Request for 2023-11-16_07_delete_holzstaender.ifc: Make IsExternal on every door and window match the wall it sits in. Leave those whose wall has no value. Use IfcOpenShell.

First a look at what the model holds.

```python
import ifcopenshell
import ifcopenshell.util.element

model = ifcopenshell.open("2023-11-16_07_delete_holzstaender.ifc")
print(model.schema)
seen = {}
for e in model.by_type("IfcDoor") + model.by_type("IfcWindow"):
    if not e.FillsVoids:
        continue
    host = e.FillsVoids[0].RelatingOpeningElement.VoidsElements[0].RelatingBuildingElement
    own = ifcopenshell.util.element.get_pset(e, f"Pset_{e.is_a()[3:].removesuffix('StandardCase')}Common", "IsExternal")
    wall = ifcopenshell.util.element.get_pset(host, "Pset_WallCommon", "IsExternal")
    seen[e.is_a(), own, wall] = seen.get((e.is_a(), own, wall), 0) + 1
for (cls, own, wall), count in sorted(seen.items(), key=str):
    print(count, cls, "IsExternal:", own, "| host wall:", wall)
```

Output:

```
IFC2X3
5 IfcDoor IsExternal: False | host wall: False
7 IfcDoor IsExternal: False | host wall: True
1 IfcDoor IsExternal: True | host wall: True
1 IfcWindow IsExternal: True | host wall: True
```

```python
import ifcopenshell
import ifcopenshell.api.pset
import ifcopenshell.util.element

model = ifcopenshell.open("2023-11-16_07_delete_holzstaender.ifc")

count = 0
for ifc_class, pset_name in (("IfcDoor", "Pset_DoorCommon"), ("IfcWindow", "Pset_WindowCommon")):
    for e in model.by_type(ifc_class):
        if not e.FillsVoids:
            continue
        host = e.FillsVoids[0].RelatingOpeningElement.VoidsElements[0].RelatingBuildingElement
        external = ifcopenshell.util.element.get_pset(host, "Pset_WallCommon", "IsExternal")
        if external is None or ifcopenshell.util.element.get_pset(e, pset_name, "IsExternal") == external:
            continue
        pset = ifcopenshell.api.pset.add_pset(model, product=e, name=pset_name)
        ifcopenshell.api.pset.edit_pset(model, pset=pset, properties={"IsExternal": external})
        count += 1

print(count, "updated")

model.write("2023-11-16_07_delete_holzstaender_edited.ifc")
```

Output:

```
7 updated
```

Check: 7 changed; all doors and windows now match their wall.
